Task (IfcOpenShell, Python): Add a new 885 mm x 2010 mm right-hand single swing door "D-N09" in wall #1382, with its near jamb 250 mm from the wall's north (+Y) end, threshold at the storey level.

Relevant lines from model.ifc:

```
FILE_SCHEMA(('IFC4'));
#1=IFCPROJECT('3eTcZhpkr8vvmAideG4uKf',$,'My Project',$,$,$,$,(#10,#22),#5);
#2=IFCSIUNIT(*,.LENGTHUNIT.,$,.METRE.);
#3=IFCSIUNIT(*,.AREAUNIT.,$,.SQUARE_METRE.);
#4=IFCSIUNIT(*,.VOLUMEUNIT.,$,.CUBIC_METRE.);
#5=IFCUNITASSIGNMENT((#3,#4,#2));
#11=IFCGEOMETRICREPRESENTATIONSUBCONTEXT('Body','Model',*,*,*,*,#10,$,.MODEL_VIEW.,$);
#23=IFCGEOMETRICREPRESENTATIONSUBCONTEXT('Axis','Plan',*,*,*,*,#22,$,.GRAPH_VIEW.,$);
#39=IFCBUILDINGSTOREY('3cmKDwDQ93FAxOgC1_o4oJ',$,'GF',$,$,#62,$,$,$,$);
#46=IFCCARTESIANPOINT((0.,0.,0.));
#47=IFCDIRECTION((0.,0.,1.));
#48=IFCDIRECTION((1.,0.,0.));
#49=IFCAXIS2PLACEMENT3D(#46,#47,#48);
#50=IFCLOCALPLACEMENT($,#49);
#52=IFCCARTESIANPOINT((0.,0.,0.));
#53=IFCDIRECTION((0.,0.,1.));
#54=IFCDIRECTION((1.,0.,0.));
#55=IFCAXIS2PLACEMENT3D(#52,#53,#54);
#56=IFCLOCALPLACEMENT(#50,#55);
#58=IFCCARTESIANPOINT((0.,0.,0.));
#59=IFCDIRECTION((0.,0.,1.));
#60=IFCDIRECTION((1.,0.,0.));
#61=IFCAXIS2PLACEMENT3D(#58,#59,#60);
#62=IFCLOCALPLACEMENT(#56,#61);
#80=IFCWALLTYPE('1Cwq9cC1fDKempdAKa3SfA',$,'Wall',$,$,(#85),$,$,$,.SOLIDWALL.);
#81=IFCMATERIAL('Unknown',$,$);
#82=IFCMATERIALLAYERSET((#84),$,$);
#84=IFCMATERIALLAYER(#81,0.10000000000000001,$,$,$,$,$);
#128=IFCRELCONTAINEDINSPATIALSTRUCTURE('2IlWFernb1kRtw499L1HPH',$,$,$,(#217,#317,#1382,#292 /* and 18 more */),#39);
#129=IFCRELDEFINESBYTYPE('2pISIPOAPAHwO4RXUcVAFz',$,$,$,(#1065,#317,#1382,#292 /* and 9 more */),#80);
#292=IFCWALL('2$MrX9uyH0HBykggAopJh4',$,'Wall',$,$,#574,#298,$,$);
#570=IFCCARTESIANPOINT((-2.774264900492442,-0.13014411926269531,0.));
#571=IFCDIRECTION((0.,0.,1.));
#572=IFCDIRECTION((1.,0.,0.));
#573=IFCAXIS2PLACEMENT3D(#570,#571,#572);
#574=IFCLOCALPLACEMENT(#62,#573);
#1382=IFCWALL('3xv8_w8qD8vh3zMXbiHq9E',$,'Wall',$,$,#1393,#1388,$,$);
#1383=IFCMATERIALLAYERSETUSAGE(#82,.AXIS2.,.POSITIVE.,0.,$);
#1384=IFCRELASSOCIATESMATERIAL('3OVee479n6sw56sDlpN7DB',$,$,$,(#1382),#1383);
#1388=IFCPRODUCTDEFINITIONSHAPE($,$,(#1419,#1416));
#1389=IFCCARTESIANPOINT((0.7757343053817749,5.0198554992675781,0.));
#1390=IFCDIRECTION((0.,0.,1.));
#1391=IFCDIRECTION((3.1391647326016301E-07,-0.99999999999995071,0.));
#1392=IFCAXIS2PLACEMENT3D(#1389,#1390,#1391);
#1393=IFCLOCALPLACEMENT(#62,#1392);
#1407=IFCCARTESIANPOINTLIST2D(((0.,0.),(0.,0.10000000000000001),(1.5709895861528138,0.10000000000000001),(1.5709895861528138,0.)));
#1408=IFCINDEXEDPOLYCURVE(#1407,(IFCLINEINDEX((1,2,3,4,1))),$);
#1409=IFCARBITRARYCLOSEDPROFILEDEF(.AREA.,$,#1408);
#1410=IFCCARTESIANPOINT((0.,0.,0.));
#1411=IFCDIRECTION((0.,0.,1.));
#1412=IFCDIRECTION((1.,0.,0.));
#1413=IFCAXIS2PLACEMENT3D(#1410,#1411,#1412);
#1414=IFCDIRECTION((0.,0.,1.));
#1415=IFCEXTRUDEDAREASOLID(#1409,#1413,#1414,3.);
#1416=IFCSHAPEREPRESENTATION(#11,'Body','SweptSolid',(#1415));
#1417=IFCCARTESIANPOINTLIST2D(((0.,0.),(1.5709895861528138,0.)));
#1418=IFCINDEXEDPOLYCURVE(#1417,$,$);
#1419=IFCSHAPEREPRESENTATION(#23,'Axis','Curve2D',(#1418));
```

```python
import numpy as np
import ifcopenshell
import ifcopenshell.api.feature
import ifcopenshell.api.geometry
import ifcopenshell.api.root
import ifcopenshell.api.spatial
import ifcopenshell.geom
import ifcopenshell.util.element
import ifcopenshell.util.placement
import ifcopenshell.util.representation
import ifcopenshell.util.shape
import ifcopenshell.util.unit

model = ifcopenshell.open("model.ifc")
unit_scale = ifcopenshell.util.unit.calculate_unit_scale(model)
settings = ifcopenshell.geom.settings()


def volume(element):
    """Net volume in cubic metres, openings subtracted."""
    shape = ifcopenshell.geom.create_shape(settings, element)
    return ifcopenshell.util.shape.get_volume(shape.geometry)


wall = model.by_guid("3xv8_w8qD8vh3zMXbiHq9E")
storey = ifcopenshell.util.element.get_container(wall, ifc_class="IfcBuildingStorey")
context = ifcopenshell.util.representation.get_context(model, "Model", "Body", "MODEL_VIEW")
before = volume(wall)

width, height, from_end, sill = 0.885, 2.01, 0.25, 0.0  # metres

# The wall runs along its own X axis, and the end named is its -X end.
wall_shape = ifcopenshell.geom.create_shape(settings, wall)
x, y, z = ifcopenshell.util.shape.get_vertices(wall_shape.geometry).T
start = x.min() + from_end
face, thickness = float(y.min()), float(y.max() - y.min())
wall_matrix = ifcopenshell.util.placement.get_local_placement(wall.ObjectPlacement)
level = ifcopenshell.util.placement.get_local_placement(storey.ObjectPlacement)[2, 3]


def in_wall(x, y):
    """Placement at x, y metres in the wall's axes, at sill height."""
    matrix = wall_matrix.copy()
    matrix[:, 3] = wall_matrix @ np.array([x / unit_scale, y / unit_scale, 0.0, 1.0])
    matrix[2, 3] = level + sill / unit_scale
    return matrix


# Opening: a box that overshoots both wall faces by 50 mm.
opening = ifcopenshell.api.root.create_entity(model, ifc_class="IfcOpeningElement", predefined_type="OPENING")
box = ifcopenshell.api.geometry.add_wall_representation(
    model, context=context, length=width, height=height, thickness=thickness + 0.1
)
ifcopenshell.api.geometry.assign_representation(model, product=opening, representation=box)
ifcopenshell.api.geometry.edit_object_placement(model, product=opening, matrix=in_wall(start, face - 0.05), is_si=False)
ifcopenshell.api.feature.add_feature(model, feature=opening, element=wall)

door = ifcopenshell.api.root.create_entity(model, ifc_class="IfcDoor", name="D-N09", predefined_type="DOOR")
door.OverallWidth, door.OverallHeight = width / unit_scale, height / unit_scale
door.OperationType = "SINGLE_SWING_RIGHT"
body = ifcopenshell.api.geometry.add_door_representation(
    model,
    context=context,
    overall_width=door.OverallWidth,
    overall_height=door.OverallHeight,
    operation_type="SINGLE_SWING_RIGHT",
    lining_properties={"LiningDepth": thickness / unit_scale, "ThresholdDepth": thickness / unit_scale},
)
ifcopenshell.api.geometry.assign_representation(model, product=door, representation=body)
ifcopenshell.api.spatial.assign_container(model, products=[door], relating_structure=storey)
ifcopenshell.api.feature.add_filling(model, opening=opening, element=door)

# The lining spans the wall, so the door starts at the wall face.
ifcopenshell.api.geometry.edit_object_placement(model, product=door, matrix=in_wall(start, face), is_si=False)

after = volume(wall)

print(f"wall volume {before:.3f} -> {after:.3f} m3")

model.write("model_updated.ifc")
```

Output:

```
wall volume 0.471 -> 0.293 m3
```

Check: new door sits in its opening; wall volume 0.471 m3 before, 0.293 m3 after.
